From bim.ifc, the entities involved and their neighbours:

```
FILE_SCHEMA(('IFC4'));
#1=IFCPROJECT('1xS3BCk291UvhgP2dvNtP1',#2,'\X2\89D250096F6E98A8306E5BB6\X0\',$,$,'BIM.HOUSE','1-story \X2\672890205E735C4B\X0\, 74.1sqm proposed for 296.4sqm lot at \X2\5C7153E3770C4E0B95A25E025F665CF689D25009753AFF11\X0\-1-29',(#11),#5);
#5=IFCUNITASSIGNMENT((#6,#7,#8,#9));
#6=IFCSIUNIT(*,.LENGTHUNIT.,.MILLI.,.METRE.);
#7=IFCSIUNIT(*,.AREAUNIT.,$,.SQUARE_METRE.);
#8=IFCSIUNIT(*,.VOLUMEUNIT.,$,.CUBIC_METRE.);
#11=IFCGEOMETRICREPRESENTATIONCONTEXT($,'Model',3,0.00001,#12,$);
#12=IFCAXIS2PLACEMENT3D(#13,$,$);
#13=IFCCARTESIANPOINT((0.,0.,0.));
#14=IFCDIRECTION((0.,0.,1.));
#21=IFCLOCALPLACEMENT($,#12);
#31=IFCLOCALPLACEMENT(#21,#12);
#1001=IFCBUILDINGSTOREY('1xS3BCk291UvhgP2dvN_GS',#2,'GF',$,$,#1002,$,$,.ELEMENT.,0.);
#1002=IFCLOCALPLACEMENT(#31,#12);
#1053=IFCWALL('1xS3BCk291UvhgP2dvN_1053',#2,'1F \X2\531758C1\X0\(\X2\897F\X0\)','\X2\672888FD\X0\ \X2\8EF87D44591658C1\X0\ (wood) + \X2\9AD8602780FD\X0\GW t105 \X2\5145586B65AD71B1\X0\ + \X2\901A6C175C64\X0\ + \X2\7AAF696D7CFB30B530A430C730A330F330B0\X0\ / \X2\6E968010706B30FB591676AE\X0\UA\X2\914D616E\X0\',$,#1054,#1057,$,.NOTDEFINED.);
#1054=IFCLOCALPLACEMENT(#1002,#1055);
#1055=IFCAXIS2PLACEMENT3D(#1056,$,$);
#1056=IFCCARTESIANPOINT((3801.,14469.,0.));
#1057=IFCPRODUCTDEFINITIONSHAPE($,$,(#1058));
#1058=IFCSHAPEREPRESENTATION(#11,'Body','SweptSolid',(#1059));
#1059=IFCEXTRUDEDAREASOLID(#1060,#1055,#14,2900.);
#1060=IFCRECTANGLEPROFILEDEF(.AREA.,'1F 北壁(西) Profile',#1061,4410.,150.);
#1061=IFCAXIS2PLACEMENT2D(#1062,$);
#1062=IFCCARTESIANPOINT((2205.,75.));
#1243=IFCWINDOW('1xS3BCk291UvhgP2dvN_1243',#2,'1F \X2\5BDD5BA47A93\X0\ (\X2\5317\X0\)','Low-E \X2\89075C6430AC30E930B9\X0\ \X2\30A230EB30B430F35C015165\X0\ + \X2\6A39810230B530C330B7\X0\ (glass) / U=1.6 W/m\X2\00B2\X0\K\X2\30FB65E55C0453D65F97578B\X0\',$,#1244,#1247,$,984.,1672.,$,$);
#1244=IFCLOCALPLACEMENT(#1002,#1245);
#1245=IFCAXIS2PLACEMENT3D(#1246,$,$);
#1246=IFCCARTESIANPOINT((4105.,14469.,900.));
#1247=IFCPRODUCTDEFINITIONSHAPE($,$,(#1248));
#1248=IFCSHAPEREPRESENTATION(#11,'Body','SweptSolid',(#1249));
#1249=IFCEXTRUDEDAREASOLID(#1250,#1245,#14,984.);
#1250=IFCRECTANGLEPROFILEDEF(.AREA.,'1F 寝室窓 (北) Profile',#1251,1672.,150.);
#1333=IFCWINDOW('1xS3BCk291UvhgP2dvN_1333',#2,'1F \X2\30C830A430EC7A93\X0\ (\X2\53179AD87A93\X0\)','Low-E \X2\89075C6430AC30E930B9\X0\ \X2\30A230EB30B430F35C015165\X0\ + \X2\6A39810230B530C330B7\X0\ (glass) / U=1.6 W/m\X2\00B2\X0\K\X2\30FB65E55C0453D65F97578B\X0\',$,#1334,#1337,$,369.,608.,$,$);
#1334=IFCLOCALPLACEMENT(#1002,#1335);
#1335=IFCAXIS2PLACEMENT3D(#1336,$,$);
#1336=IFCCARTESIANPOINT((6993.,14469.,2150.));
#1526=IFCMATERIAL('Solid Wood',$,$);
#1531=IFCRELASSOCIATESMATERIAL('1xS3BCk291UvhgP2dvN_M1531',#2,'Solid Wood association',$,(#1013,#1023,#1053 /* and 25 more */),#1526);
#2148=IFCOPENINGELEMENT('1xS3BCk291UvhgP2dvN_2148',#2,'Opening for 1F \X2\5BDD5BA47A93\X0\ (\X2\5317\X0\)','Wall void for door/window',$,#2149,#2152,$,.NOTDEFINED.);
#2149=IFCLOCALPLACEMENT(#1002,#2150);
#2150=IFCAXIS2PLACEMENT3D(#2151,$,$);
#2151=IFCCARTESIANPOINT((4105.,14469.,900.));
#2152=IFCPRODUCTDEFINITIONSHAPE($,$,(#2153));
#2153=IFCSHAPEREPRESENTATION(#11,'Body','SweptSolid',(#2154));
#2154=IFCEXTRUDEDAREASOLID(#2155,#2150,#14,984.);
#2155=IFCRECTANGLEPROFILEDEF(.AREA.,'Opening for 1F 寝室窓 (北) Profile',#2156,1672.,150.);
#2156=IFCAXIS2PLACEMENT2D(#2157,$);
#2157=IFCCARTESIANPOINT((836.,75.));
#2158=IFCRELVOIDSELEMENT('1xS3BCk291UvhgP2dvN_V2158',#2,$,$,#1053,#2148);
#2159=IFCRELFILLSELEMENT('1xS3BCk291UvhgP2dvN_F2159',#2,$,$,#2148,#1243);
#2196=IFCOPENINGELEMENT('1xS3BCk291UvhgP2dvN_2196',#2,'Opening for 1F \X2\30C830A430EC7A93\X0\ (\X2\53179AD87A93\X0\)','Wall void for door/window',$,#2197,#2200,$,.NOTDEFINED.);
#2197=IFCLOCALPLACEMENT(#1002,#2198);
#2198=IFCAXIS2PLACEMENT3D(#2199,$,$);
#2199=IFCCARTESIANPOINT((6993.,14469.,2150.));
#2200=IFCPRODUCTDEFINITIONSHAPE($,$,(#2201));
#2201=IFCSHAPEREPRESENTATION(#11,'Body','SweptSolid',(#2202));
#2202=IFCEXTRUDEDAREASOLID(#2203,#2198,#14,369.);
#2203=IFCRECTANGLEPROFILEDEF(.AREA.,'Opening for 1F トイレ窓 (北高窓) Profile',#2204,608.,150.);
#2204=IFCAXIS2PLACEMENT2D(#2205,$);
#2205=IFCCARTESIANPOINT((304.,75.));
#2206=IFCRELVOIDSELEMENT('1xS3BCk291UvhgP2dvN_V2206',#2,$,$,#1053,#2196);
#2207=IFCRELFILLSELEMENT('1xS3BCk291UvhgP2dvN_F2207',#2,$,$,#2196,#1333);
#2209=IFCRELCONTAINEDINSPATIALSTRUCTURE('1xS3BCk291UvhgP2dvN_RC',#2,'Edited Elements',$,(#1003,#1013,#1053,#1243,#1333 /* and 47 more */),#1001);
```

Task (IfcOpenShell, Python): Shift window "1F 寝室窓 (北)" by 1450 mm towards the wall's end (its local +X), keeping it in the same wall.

```python
import ifcopenshell
import ifcopenshell.api.geometry
import ifcopenshell.util.placement
import ifcopenshell.util.unit

model = ifcopenshell.open("bim.ifc")
unit_scale = ifcopenshell.util.unit.calculate_unit_scale(model)

window = model.by_guid("1xS3BCk291UvhgP2dvN_1243")
opening = window.FillsVoids[0].RelatingOpeningElement
wall = opening.VoidsElements[0].RelatingBuildingElement

wall_matrix = ifcopenshell.util.placement.get_local_placement(wall.ObjectPlacement)
shift = wall_matrix[:3, 0] * 1.45 / unit_scale
before = ifcopenshell.util.placement.get_local_placement(window.ObjectPlacement)[:3, 3].copy()

# The window is not placed relative to its opening, so move both.
for product in (opening, window):
    matrix = ifcopenshell.util.placement.get_local_placement(product.ObjectPlacement)
    matrix[:3, 3] += shift
    ifcopenshell.api.geometry.edit_object_placement(model, product=product, matrix=matrix, is_si=False)

after = ifcopenshell.util.placement.get_local_placement(window.ObjectPlacement)[:3, 3]
print("window moved by", (after - before).round(3) + 0.0)

model.write("bim_v2.ifc")
```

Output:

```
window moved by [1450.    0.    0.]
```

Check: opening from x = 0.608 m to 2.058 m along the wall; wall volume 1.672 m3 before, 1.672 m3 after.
